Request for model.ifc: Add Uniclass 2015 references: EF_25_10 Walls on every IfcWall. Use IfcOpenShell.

First a look at what the model holds.

```python
import ifcopenshell

model = ifcopenshell.open("model.ifc")
print(model.schema)
print("classifications:", [c.Name for c in model.by_type("IfcClassification")])
for ifc_class in ("IfcDoor", "IfcRoof", "IfcStair", "IfcWall", "IfcWindow"):
    print(ifc_class, len(model.by_type(ifc_class)))
```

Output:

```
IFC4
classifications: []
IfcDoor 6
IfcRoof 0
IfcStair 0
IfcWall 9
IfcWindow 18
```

```python
import ifcopenshell
import ifcopenshell.api.classification

model = ifcopenshell.open("model.ifc")

system = ifcopenshell.api.classification.add_classification(model, classification="Uniclass 2015")

codes = {
    "IfcWall": ("EF_25_10", "Walls"),
}
for ifc_class, (code, name) in codes.items():
    products = model.by_type(ifc_class)
    ifcopenshell.api.classification.add_reference(
        model, products=products, classification=system, identification=code, name=name
    )
    print(code, len(products))

model.write("model_edited.ifc")
```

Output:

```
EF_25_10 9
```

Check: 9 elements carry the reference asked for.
